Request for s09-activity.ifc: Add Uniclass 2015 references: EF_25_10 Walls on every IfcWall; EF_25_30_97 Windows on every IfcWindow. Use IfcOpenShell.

First a look at what the model holds.

```python
import ifcopenshell

model = ifcopenshell.open("s09-activity.ifc")
print(model.schema)
print("classifications:", [c.Name for c in model.by_type("IfcClassification")])
for ifc_class in ("IfcDoor", "IfcRoof", "IfcStair", "IfcWall", "IfcWindow"):
    print(ifc_class, len(model.by_type(ifc_class)))
```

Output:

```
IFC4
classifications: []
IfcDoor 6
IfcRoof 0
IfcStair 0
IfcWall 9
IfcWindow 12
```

```python
import ifcopenshell
import ifcopenshell.api.classification

model = ifcopenshell.open("s09-activity.ifc")

system = ifcopenshell.api.classification.add_classification(model, classification="Uniclass 2015")

codes = {
    "IfcWall": ("EF_25_10", "Walls"),
    "IfcWindow": ("EF_25_30_97", "Windows"),
}
for ifc_class, (code, name) in codes.items():
    products = model.by_type(ifc_class)
    ifcopenshell.api.classification.add_reference(
        model, products=products, classification=system, identification=code, name=name
    )
    print(code, len(products))

model.write("s09-activity_rev.ifc")
```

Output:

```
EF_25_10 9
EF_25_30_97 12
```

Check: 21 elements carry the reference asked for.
